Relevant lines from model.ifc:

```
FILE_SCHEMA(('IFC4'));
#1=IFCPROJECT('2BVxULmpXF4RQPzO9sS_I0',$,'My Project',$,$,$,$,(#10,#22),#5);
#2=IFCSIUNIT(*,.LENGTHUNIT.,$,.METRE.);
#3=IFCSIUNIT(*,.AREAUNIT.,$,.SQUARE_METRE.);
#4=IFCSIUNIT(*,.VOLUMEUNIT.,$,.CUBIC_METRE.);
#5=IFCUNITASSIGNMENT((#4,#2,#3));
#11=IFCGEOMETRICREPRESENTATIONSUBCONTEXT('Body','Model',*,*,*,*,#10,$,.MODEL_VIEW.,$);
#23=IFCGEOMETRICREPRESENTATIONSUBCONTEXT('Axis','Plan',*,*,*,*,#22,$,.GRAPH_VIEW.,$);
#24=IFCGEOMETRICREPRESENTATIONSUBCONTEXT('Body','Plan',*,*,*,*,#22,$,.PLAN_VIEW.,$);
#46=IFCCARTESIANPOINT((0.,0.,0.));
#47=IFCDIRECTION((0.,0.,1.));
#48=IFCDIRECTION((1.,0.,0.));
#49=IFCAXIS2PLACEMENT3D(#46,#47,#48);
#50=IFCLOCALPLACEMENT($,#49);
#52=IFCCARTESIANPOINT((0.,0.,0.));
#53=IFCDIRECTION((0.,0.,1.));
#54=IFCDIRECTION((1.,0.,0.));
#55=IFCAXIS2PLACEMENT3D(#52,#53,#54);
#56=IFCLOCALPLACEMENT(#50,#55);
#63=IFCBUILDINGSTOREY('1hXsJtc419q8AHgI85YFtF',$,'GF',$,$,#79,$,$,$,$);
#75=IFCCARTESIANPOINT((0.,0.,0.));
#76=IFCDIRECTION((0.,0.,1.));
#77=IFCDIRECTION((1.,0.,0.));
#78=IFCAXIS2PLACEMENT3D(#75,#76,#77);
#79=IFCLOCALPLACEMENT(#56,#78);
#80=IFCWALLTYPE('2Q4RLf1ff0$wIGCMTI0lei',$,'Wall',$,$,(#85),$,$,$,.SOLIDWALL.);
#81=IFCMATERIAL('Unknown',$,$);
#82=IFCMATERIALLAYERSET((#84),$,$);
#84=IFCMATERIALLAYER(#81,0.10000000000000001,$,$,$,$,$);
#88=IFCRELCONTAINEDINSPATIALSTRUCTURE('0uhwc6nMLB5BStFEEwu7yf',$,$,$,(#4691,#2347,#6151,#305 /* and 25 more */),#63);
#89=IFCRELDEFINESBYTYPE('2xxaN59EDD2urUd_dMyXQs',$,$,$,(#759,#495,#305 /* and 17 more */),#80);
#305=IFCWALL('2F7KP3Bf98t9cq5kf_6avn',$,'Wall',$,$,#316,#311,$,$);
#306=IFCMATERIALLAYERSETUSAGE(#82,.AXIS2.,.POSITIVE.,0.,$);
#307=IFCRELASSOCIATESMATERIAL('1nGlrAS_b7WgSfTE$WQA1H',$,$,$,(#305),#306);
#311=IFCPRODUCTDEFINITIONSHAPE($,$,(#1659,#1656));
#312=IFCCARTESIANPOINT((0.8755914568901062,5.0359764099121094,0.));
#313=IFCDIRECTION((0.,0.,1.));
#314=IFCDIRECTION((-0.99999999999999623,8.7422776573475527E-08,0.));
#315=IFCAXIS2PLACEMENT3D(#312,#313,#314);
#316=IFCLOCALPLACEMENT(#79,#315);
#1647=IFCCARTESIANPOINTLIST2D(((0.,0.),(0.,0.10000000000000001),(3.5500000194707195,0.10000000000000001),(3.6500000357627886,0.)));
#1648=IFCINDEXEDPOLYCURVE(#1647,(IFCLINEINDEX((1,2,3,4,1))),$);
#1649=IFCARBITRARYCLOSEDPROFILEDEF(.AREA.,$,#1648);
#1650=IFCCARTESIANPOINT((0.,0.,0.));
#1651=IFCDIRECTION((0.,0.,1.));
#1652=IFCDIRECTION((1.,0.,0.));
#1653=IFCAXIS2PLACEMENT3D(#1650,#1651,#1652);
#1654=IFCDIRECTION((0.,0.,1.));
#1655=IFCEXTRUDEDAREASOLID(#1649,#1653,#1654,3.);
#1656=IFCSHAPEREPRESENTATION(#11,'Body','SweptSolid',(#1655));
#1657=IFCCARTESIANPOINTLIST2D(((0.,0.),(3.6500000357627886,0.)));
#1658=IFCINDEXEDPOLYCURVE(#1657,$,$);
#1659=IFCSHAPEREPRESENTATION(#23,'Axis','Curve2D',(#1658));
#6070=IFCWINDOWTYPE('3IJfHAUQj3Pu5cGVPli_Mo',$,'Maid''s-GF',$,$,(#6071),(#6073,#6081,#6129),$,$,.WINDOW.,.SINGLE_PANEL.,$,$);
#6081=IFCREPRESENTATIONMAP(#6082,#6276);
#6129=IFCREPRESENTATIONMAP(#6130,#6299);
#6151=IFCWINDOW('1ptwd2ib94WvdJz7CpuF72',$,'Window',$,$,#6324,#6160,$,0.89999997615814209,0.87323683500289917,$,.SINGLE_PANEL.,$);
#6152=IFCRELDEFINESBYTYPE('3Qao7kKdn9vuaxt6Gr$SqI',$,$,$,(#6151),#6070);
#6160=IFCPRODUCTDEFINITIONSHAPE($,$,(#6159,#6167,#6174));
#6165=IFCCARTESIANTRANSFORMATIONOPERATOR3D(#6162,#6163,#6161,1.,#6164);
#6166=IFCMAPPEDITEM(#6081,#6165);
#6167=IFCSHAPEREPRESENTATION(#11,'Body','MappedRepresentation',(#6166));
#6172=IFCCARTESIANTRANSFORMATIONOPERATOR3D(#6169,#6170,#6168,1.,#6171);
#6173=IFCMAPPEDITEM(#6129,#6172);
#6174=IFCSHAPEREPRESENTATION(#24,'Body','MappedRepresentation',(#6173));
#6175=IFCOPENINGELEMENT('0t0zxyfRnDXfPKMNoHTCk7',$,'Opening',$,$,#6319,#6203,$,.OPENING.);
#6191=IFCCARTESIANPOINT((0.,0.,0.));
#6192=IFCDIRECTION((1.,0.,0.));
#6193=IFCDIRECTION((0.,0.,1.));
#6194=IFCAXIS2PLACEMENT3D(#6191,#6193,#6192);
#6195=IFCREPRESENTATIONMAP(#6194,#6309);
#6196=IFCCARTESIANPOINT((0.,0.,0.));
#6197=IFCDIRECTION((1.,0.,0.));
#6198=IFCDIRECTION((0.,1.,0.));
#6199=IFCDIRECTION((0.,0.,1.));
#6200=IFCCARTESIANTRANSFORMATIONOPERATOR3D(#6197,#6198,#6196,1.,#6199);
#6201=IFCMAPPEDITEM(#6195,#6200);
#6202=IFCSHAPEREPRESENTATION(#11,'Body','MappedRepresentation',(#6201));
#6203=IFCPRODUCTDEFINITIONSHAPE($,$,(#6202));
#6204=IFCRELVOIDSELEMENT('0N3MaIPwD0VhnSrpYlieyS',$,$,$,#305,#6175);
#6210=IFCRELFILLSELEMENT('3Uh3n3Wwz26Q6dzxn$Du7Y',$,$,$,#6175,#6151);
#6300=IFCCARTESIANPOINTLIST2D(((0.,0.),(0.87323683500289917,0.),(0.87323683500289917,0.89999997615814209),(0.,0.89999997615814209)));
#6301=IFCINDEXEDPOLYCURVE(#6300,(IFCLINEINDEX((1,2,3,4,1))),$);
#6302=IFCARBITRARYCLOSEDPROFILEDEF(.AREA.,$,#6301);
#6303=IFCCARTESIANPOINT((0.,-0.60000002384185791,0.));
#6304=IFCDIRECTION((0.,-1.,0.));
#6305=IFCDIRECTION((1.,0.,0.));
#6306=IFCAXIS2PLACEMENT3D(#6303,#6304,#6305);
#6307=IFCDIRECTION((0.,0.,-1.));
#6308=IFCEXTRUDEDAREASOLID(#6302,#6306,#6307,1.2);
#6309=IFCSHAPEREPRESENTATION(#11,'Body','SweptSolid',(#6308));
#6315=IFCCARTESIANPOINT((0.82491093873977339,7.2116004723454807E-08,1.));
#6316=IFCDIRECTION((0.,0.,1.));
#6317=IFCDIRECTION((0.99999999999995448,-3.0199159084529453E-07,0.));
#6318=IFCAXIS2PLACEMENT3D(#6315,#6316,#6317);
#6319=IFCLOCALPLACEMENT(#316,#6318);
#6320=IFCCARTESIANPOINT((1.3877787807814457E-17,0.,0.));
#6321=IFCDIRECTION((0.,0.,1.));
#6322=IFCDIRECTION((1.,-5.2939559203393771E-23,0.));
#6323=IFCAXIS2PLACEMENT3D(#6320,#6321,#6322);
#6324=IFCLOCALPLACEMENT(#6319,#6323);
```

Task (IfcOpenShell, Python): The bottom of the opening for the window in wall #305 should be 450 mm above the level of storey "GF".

```python
import numpy as np
import ifcopenshell
import ifcopenshell.api.geometry
import ifcopenshell.geom
import ifcopenshell.util.element
import ifcopenshell.util.placement
import ifcopenshell.util.shape
import ifcopenshell.util.unit

model = ifcopenshell.open("model.ifc")
unit_scale = ifcopenshell.util.unit.calculate_unit_scale(model)

window = model.by_id(6151)
opening = window.FillsVoids[0].RelatingOpeningElement
storey = ifcopenshell.util.element.get_container(window, ifc_class="IfcBuildingStorey")
level = ifcopenshell.util.placement.get_local_placement(storey.ObjectPlacement)[2, 3]

# The opening's origin need not be at the sill, so measure its lowest point.
shape = ifcopenshell.geom.create_shape(ifcopenshell.geom.settings(), opening)
bottom = ifcopenshell.util.shape.get_shape_bottom_elevation(shape, shape.geometry) / unit_scale
dz = level + 0.45 / unit_scale - bottom

shift = np.array([0.0, 0.0, dz])
# The window is placed relative to its opening, so it follows when the opening moves.
matrix = ifcopenshell.util.placement.get_local_placement(opening.ObjectPlacement)
matrix[:3, 3] += shift
ifcopenshell.api.geometry.edit_object_placement(
    model, product=opening, matrix=matrix, is_si=False, should_transform_children=True
)

print(f"moved by {dz * unit_scale:+.3f} m")

model.write("model_updated.ifc")
```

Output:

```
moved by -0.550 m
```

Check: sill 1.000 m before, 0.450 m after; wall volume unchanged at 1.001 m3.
